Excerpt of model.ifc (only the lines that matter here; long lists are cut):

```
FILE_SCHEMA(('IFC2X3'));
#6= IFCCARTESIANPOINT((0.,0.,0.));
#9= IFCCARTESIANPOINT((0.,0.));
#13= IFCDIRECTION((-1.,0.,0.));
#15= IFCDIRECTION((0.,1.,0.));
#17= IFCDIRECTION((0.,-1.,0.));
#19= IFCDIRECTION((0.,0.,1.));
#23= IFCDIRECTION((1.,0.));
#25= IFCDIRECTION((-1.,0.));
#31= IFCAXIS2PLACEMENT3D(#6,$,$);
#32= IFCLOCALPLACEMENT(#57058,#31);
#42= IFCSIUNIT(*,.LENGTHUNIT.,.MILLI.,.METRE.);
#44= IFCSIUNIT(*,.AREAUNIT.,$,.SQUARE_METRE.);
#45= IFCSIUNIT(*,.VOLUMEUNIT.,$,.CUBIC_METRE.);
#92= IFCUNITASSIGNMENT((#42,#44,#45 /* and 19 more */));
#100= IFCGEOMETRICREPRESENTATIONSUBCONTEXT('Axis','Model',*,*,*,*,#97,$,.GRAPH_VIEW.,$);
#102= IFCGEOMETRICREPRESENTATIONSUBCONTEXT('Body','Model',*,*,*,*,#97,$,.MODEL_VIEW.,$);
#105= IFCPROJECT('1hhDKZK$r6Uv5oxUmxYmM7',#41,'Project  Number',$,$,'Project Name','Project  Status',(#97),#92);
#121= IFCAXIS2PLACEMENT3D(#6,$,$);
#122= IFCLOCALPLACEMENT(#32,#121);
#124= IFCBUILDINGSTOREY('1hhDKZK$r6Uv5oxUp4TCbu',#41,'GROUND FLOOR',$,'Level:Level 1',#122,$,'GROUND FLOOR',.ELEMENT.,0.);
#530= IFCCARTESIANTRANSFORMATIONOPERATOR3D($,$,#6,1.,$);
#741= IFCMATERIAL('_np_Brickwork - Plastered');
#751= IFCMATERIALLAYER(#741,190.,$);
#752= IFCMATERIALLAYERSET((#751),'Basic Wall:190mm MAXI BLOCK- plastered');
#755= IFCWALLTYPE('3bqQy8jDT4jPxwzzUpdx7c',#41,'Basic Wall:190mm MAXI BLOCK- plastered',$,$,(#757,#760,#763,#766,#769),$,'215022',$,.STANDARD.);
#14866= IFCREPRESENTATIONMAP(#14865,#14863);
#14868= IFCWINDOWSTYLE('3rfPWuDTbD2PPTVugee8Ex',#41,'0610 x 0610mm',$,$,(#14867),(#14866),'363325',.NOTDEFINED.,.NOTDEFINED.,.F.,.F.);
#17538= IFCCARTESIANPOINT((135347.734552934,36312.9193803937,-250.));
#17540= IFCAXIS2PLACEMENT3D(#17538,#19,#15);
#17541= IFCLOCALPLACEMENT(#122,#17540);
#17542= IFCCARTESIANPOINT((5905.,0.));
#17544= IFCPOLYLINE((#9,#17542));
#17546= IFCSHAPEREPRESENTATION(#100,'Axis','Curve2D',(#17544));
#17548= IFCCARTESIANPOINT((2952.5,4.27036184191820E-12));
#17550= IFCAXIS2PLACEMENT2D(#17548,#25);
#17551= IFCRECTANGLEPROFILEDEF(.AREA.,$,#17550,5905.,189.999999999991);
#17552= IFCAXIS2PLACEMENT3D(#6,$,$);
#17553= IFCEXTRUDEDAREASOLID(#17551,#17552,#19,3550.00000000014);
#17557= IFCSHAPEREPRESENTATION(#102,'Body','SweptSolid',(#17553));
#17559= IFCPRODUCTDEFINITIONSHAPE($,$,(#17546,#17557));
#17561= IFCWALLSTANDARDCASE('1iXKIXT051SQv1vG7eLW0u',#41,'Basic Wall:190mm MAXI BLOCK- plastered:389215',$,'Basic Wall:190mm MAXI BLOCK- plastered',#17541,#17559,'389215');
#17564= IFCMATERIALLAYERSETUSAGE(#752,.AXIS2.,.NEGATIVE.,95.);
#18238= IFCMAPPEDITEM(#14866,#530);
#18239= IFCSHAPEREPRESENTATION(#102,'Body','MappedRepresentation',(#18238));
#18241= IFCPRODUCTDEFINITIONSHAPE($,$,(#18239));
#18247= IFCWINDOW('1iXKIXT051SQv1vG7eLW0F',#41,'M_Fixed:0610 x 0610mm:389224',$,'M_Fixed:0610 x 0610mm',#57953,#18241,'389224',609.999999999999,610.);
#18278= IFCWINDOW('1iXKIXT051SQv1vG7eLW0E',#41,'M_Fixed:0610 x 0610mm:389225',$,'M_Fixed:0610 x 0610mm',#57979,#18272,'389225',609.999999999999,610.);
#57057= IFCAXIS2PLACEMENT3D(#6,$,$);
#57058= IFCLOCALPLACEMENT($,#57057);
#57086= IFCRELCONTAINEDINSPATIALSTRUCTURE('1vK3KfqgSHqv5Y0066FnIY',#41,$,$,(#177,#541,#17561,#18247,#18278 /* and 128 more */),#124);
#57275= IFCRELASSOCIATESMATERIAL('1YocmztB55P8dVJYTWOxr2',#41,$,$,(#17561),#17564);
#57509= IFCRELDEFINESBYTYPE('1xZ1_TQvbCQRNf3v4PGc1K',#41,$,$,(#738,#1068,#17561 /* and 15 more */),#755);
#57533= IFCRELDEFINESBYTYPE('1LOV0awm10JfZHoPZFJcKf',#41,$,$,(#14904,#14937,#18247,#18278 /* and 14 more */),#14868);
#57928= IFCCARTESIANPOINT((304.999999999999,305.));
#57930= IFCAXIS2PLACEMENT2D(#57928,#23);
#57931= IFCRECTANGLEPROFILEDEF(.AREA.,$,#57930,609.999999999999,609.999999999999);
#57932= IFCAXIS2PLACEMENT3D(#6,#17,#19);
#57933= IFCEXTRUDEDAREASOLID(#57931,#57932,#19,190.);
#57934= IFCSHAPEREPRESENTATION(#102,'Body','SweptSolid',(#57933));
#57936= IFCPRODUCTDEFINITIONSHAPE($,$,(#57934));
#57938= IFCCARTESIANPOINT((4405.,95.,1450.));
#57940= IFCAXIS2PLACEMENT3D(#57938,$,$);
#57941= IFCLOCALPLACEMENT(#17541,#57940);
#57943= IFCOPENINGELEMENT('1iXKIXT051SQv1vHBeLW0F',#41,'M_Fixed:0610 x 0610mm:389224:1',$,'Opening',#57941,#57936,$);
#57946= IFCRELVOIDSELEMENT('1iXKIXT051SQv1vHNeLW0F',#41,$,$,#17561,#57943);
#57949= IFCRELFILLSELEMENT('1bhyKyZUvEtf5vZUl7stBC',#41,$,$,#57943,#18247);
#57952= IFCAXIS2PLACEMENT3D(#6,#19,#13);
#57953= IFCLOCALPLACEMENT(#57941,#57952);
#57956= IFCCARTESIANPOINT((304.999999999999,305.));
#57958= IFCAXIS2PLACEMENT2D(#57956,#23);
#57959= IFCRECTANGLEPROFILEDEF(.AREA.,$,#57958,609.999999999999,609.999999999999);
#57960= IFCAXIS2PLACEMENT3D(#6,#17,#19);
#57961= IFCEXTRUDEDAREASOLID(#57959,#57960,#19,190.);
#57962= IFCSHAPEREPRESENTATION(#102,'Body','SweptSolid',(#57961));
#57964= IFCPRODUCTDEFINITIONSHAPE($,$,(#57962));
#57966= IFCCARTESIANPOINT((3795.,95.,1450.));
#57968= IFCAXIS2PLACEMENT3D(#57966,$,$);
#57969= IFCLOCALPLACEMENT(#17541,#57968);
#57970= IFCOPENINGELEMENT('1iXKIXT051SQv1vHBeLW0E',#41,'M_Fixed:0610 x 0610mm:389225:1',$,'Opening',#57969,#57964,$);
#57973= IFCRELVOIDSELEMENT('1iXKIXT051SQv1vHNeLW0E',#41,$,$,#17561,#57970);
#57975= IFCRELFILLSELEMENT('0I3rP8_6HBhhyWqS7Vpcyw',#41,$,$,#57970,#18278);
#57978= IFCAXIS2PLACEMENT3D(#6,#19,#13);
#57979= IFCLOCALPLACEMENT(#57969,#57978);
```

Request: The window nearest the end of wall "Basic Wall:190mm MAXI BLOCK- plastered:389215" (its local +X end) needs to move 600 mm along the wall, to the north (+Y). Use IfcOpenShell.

```python
import ifcopenshell
import ifcopenshell.api.geometry
import ifcopenshell.util.placement
import ifcopenshell.util.unit

model = ifcopenshell.open("model.ifc")
unit_scale = ifcopenshell.util.unit.calculate_unit_scale(model)

window = model.by_id(18247)
opening = window.FillsVoids[0].RelatingOpeningElement
wall = opening.VoidsElements[0].RelatingBuildingElement

wall_matrix = ifcopenshell.util.placement.get_local_placement(wall.ObjectPlacement)
shift = wall_matrix[:3, 0] * 0.6 / unit_scale
before = ifcopenshell.util.placement.get_local_placement(window.ObjectPlacement)[:3, 3].copy()

# The window is placed relative to its opening, so it follows when the opening moves.
matrix = ifcopenshell.util.placement.get_local_placement(opening.ObjectPlacement)
matrix[:3, 3] += shift
ifcopenshell.api.geometry.edit_object_placement(
    model, product=opening, matrix=matrix, is_si=False, should_transform_children=True
)

after = ifcopenshell.util.placement.get_local_placement(window.ObjectPlacement)[:3, 3]
print("window moved by", (after - before).round(3) + 0.0)

model.write("model_updated.ifc")
```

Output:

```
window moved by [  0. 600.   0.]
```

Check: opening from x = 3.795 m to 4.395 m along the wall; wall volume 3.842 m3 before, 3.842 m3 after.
